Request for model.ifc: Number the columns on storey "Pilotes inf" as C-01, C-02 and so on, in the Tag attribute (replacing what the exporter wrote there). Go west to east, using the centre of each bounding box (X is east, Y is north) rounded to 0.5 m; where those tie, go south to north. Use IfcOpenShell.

First a look at what the model holds.

```python
import ifcopenshell
import ifcopenshell.util.element
import ifcopenshell.util.placement

model = ifcopenshell.open("model.ifc")
print(model.schema)
storey = next(s for s in model.by_type("IfcBuildingStorey") if s.Name == "Pilotes inf")
columns = [e for e in ifcopenshell.util.element.get_decomposition(storey) if e.is_a("IfcColumn")]
for e in sorted(columns, key=lambda e: e.id()):
    origin = ifcopenshell.util.placement.get_local_placement(e.ObjectPlacement)[:3, 3]
    print(e.id(), e.Tag, e.Name, origin.round(2) + 0.0, sep=" | ")
```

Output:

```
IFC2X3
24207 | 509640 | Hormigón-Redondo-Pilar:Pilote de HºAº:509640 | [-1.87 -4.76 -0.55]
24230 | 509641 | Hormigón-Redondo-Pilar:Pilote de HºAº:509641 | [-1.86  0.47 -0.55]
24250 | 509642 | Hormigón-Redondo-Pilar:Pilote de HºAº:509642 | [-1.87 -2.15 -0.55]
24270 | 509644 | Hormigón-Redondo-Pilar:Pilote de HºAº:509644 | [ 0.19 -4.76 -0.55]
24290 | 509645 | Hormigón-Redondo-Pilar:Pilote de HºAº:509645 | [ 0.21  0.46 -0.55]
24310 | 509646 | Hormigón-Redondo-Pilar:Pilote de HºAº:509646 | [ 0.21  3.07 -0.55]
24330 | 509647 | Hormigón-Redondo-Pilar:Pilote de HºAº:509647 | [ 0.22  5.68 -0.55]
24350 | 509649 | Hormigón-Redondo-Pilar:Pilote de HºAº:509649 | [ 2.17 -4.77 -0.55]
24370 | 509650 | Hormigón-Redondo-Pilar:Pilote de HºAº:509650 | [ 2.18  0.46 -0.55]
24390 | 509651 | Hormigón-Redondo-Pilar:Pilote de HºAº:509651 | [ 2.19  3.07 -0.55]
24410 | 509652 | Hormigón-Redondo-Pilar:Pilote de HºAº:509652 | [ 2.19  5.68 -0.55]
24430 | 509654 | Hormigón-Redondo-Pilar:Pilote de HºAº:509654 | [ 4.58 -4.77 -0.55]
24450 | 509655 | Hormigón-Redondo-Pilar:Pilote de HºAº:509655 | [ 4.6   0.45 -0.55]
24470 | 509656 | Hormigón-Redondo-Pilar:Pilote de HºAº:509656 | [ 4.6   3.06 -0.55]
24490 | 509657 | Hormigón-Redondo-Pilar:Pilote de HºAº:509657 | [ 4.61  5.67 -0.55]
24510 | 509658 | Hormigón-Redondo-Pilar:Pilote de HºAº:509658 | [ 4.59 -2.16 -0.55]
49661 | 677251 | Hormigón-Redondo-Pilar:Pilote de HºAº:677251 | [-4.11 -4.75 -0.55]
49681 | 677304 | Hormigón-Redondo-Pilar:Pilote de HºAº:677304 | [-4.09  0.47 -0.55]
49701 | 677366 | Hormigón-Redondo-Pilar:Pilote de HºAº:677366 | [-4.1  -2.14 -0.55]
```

```python
import ifcopenshell
import ifcopenshell.geom
import ifcopenshell.util.element
import ifcopenshell.util.shape

model = ifcopenshell.open("model.ifc")
settings = ifcopenshell.geom.settings()
settings.set("use-world-coords", True)


def centre(element):
    shape = ifcopenshell.geom.create_shape(settings, element)
    return ifcopenshell.util.shape.get_bbox_centroid(shape.geometry)


storey = next(s for s in model.by_type("IfcBuildingStorey") if s.Name == "Pilotes inf")
columns = [e for e in ifcopenshell.util.element.get_decomposition(storey) if e.is_a("IfcColumn")]

# Insertion points can sit at a corner or the storey origin, so sort by the geometry (in metres).
centres = {e: centre(e) for e in columns}
columns.sort(key=lambda e: (round(centres[e][0] / 0.5), centres[e][1]))

for i, e in enumerate(columns, start=1):
    number = f"C-{i:02d}"
    e.Tag = number
    print(e.id(), number)

model.write("model_v2.ifc")
```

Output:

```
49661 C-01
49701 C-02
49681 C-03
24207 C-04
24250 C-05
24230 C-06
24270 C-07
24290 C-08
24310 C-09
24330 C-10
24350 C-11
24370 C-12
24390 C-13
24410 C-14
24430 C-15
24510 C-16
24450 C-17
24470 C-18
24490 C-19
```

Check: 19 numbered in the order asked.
